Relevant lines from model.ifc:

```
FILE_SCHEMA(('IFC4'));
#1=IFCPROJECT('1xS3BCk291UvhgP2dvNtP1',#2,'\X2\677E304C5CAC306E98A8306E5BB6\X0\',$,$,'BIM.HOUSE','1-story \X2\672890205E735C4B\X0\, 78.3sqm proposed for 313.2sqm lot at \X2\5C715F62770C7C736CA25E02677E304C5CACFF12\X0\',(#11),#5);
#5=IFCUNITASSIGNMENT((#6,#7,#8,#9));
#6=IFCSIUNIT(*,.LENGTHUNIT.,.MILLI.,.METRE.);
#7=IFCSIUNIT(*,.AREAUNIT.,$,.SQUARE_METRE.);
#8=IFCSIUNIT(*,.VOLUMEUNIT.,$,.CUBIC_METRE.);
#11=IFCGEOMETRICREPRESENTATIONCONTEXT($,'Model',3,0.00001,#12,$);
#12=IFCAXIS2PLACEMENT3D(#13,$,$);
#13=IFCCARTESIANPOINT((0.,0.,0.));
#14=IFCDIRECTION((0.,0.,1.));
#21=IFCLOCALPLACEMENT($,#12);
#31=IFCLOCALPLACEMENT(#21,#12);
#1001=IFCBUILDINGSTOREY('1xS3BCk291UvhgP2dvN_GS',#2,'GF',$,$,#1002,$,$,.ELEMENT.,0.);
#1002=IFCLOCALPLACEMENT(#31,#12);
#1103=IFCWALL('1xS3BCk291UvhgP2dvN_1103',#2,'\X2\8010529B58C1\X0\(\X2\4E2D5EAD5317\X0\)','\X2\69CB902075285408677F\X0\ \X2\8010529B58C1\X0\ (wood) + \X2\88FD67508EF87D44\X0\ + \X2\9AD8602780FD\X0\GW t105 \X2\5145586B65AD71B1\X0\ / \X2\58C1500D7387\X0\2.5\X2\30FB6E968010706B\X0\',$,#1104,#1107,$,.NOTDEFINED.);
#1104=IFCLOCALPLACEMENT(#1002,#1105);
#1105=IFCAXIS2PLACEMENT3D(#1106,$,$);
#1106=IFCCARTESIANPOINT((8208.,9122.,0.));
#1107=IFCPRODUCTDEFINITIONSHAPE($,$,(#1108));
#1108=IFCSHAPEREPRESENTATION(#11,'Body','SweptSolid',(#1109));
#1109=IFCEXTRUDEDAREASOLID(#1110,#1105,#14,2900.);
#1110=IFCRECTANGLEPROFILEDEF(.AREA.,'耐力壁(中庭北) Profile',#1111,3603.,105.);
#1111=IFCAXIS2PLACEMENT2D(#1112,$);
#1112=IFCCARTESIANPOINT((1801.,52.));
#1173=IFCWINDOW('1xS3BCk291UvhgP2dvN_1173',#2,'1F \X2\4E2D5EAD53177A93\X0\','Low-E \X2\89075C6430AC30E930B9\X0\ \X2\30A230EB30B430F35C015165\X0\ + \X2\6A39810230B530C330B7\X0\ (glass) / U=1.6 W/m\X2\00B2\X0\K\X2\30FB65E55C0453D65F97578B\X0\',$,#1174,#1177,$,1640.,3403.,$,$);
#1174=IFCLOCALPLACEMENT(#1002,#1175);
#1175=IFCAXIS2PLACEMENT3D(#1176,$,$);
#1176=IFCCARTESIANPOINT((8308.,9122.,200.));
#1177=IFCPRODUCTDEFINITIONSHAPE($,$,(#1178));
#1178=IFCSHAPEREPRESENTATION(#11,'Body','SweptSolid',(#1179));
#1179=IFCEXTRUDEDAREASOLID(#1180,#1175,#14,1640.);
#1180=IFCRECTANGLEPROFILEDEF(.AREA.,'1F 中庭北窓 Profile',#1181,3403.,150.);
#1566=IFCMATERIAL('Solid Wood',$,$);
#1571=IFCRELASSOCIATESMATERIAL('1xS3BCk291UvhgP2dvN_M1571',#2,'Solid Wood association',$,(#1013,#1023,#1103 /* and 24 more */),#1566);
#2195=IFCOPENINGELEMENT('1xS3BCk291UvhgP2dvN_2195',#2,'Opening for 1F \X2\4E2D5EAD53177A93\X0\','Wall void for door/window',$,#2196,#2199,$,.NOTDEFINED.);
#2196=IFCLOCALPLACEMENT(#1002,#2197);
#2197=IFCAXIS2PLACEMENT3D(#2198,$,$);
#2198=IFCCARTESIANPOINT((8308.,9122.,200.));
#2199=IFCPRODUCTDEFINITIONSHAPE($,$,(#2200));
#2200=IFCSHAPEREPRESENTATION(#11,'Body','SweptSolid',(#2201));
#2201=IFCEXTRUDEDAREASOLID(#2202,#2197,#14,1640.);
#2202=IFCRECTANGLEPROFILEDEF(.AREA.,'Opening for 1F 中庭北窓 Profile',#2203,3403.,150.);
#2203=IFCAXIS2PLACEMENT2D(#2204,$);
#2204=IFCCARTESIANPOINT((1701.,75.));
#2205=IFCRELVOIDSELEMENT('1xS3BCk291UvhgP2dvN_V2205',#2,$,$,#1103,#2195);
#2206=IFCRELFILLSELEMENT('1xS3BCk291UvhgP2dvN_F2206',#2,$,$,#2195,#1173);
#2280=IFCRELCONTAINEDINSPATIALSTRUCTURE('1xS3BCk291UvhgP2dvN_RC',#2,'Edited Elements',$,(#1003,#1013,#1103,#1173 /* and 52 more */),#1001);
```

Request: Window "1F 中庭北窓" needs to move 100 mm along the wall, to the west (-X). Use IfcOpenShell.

```python
import ifcopenshell
import ifcopenshell.api.geometry
import ifcopenshell.util.placement
import ifcopenshell.util.unit

model = ifcopenshell.open("model.ifc")
unit_scale = ifcopenshell.util.unit.calculate_unit_scale(model)

window = model.by_guid("1xS3BCk291UvhgP2dvN_1173")
opening = window.FillsVoids[0].RelatingOpeningElement
wall = opening.VoidsElements[0].RelatingBuildingElement

wall_matrix = ifcopenshell.util.placement.get_local_placement(wall.ObjectPlacement)
shift = wall_matrix[:3, 0] * -0.1 / unit_scale
before = ifcopenshell.util.placement.get_local_placement(window.ObjectPlacement)[:3, 3].copy()

# The window is not placed relative to its opening, so move both.
for product in (opening, window):
    matrix = ifcopenshell.util.placement.get_local_placement(product.ObjectPlacement)
    matrix[:3, 3] += shift
    ifcopenshell.api.geometry.edit_object_placement(model, product=product, matrix=matrix, is_si=False)

after = ifcopenshell.util.placement.get_local_placement(window.ObjectPlacement)[:3, 3]
print("window moved by", (after - before).round(3) + 0.0)

model.write("model_edited.ifc")
```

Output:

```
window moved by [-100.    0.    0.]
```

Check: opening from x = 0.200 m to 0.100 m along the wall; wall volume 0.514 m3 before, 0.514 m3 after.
